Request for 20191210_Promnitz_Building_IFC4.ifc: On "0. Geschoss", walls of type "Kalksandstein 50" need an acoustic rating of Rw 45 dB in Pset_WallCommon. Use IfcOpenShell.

First a look at what the model holds.

```python
import ifcopenshell
import ifcopenshell.util.element

model = ifcopenshell.open("20191210_Promnitz_Building_IFC4.ifc")
print(model.schema)
storey = next(s for s in model.by_type("IfcBuildingStorey") if s.Name == "0. Geschoss")
walls = [e for e in ifcopenshell.util.element.get_decomposition(storey) if e.is_a("IfcWall")]
seen = {}
for e in walls:
    element_type = ifcopenshell.util.element.get_type(e)
    key = (element_type.Name if element_type != e and element_type else None, ifcopenshell.util.element.get_pset(e, "Pset_WallCommon", "AcousticRating"))
    seen[key] = seen.get(key, 0) + 1
for (name, value), count in sorted(seen.items(), key=str):
    print(count, "x", name, "|", value)
```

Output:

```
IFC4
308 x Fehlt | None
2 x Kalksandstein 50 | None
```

```python
import ifcopenshell
import ifcopenshell.api.pset
import ifcopenshell.util.element

model = ifcopenshell.open("20191210_Promnitz_Building_IFC4.ifc")

storey = next(s for s in model.by_type("IfcBuildingStorey") if s.Name == "0. Geschoss")
walls = [e for e in ifcopenshell.util.element.get_decomposition(storey) if e.is_a("IfcWall")]

count = 0
for e in walls:
    element_type = ifcopenshell.util.element.get_type(e)
    if element_type in (None, e) or element_type.Name != "Kalksandstein 50":
        continue
    # add_pset returns the element's existing set when there is one.
    pset = ifcopenshell.api.pset.add_pset(model, product=e, name="Pset_WallCommon")
    ifcopenshell.api.pset.edit_pset(model, pset=pset, properties={"AcousticRating": "Rw 45 dB"})
    count += 1

print(count, "walls updated")

model.write("20191210_Promnitz_Building_IFC4-out.ifc")
```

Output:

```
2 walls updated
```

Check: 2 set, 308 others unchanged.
